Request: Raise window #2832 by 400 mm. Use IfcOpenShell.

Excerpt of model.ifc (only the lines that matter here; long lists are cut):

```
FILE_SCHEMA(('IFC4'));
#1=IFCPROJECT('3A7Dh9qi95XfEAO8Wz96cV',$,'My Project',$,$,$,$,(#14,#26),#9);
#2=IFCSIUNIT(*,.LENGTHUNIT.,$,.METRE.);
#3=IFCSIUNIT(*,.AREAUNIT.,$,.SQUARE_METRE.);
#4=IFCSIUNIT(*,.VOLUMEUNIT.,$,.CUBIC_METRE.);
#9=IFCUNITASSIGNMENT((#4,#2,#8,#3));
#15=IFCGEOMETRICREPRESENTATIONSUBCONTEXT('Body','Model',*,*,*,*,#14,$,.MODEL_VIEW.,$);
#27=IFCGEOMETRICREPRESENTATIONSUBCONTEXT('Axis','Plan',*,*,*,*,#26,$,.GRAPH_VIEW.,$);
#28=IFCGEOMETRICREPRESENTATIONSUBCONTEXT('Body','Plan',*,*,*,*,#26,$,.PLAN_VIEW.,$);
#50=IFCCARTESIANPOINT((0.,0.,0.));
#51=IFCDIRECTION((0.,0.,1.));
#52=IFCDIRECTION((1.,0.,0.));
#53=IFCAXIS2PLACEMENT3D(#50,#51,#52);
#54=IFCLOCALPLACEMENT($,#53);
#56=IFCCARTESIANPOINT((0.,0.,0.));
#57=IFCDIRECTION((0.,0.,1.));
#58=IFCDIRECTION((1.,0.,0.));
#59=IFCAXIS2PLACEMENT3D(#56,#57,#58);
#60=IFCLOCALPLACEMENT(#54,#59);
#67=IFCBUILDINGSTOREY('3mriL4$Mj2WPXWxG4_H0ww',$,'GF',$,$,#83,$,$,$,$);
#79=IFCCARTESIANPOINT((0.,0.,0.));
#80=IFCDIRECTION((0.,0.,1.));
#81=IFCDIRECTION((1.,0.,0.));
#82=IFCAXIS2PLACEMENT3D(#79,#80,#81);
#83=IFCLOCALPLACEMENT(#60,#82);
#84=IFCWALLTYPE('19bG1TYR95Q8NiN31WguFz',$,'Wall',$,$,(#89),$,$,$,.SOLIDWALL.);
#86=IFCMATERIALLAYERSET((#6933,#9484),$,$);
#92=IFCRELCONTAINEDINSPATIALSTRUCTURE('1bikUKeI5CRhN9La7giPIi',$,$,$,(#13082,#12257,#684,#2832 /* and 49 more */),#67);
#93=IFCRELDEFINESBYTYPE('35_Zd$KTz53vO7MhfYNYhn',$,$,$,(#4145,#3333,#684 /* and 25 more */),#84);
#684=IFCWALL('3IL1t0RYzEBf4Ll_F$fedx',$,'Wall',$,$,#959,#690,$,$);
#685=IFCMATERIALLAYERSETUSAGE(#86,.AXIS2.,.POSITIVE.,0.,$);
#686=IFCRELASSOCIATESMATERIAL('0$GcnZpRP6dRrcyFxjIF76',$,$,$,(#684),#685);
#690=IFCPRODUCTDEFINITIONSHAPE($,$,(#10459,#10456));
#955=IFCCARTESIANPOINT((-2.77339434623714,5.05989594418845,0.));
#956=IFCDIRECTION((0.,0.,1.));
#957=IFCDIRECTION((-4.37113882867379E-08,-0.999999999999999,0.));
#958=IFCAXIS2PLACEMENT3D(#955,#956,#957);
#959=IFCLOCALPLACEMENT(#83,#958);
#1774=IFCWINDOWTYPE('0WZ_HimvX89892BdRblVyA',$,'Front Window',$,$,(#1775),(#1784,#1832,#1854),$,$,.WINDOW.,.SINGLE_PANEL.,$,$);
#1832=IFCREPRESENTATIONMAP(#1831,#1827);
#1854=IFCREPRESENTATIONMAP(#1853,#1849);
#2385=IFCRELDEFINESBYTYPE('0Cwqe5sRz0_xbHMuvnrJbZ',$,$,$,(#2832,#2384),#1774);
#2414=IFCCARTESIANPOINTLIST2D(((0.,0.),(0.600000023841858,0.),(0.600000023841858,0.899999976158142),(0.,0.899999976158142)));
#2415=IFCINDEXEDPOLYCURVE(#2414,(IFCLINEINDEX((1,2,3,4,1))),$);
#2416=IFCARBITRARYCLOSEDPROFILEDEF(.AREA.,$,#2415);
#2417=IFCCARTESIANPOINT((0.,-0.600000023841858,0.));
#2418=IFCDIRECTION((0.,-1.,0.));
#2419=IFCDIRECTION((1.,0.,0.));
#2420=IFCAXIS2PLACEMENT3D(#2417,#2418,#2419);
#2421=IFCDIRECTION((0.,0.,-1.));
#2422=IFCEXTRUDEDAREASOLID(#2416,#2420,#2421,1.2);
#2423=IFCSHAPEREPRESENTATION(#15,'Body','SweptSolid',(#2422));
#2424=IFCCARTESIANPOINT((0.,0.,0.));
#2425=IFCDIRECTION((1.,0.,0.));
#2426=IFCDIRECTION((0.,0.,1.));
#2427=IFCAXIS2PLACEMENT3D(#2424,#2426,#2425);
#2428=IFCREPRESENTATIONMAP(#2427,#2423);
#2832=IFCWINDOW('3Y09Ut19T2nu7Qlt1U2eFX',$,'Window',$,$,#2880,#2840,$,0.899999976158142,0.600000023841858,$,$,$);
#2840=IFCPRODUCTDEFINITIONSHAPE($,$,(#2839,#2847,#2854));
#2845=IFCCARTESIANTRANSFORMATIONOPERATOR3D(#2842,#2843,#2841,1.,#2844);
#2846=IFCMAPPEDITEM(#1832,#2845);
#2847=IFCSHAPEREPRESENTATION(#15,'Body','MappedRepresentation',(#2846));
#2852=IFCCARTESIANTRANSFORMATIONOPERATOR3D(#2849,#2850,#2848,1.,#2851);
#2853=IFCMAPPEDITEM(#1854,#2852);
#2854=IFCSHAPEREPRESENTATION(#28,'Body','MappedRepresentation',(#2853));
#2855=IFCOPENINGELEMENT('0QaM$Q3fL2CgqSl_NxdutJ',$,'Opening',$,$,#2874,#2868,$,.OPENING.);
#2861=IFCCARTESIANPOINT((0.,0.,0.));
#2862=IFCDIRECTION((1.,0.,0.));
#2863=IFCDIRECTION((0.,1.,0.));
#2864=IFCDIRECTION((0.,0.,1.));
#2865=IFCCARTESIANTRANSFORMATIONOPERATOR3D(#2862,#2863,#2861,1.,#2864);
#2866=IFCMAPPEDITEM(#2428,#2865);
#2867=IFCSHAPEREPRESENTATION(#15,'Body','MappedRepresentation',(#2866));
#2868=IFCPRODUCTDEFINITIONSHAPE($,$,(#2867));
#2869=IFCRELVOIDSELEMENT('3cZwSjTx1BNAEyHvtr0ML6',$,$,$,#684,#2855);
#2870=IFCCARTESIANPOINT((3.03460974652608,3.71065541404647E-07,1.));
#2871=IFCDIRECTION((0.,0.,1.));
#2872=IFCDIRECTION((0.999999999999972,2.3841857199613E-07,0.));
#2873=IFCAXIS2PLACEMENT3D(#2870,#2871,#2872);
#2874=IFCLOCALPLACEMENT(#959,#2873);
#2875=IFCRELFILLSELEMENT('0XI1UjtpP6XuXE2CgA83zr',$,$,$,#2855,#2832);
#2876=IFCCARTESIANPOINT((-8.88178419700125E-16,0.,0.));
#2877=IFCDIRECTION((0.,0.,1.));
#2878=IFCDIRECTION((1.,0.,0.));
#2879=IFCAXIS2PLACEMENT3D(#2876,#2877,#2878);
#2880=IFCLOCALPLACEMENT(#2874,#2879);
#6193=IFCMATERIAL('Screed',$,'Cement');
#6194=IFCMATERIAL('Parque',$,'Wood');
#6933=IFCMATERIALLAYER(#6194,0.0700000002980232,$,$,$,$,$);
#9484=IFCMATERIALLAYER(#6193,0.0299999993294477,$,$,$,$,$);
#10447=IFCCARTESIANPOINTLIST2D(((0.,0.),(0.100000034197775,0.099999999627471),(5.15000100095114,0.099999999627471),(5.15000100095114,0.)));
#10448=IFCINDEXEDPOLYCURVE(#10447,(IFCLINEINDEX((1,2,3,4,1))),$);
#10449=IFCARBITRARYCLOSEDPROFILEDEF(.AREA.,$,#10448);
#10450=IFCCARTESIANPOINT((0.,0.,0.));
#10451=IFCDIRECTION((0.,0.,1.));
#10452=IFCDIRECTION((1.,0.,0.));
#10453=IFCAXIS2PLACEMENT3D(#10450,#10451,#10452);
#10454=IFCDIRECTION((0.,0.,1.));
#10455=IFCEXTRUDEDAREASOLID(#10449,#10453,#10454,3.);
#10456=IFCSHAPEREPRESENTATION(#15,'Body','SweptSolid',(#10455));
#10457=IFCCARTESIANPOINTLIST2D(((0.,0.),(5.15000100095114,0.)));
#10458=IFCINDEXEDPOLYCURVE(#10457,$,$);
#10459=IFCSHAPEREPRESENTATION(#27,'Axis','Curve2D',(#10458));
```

```python
import numpy as np
import ifcopenshell
import ifcopenshell.api.geometry
import ifcopenshell.util.placement
import ifcopenshell.util.unit

model = ifcopenshell.open("model.ifc")
unit_scale = ifcopenshell.util.unit.calculate_unit_scale(model)

window = model.by_guid("3Y09Ut19T2nu7Qlt1U2eFX")
opening = window.FillsVoids[0].RelatingOpeningElement
dz = 0.4 / unit_scale

shift = np.array([0.0, 0.0, dz])
# The window is placed relative to its opening, so it follows when the opening moves.
matrix = ifcopenshell.util.placement.get_local_placement(opening.ObjectPlacement)
matrix[:3, 3] += shift
ifcopenshell.api.geometry.edit_object_placement(
    model, product=opening, matrix=matrix, is_si=False, should_transform_children=True
)

print(f"moved by {dz * unit_scale:+.3f} m")

model.write("model_v2.ifc")
```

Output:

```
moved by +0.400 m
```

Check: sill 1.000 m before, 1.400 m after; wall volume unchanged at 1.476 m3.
